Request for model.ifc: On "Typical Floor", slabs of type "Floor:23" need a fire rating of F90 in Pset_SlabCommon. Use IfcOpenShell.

First a look at what the model holds.

```python
import ifcopenshell
import ifcopenshell.util.element

model = ifcopenshell.open("model.ifc")
print(model.schema)
storey = next(s for s in model.by_type("IfcBuildingStorey") if s.Name == "Typical Floor")
slabs = [e for e in ifcopenshell.util.element.get_decomposition(storey) if e.is_a("IfcSlab")]
seen = {}
for e in slabs:
    element_type = ifcopenshell.util.element.get_type(e)
    key = (element_type.Name if element_type != e and element_type else None, ifcopenshell.util.element.get_pset(e, "Pset_SlabCommon", "FireRating"))
    seen[key] = seen.get(key, 0) + 1
for (name, value), count in sorted(seen.items(), key=str):
    print(count, "x", name, "|", value)
```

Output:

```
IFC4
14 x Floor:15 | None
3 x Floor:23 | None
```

```python
import ifcopenshell
import ifcopenshell.api.pset
import ifcopenshell.util.element

model = ifcopenshell.open("model.ifc")

storey = next(s for s in model.by_type("IfcBuildingStorey") if s.Name == "Typical Floor")
slabs = [e for e in ifcopenshell.util.element.get_decomposition(storey) if e.is_a("IfcSlab")]

count = 0
for e in slabs:
    element_type = ifcopenshell.util.element.get_type(e)
    if element_type in (None, e) or element_type.Name != "Floor:23":
        continue
    # add_pset returns the element's existing set when there is one.
    pset = ifcopenshell.api.pset.add_pset(model, product=e, name="Pset_SlabCommon")
    ifcopenshell.api.pset.edit_pset(model, pset=pset, properties={"FireRating": "F90"})
    count += 1

print(count, "slabs updated")

model.write("model_rev.ifc")
```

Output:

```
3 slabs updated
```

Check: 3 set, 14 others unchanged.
